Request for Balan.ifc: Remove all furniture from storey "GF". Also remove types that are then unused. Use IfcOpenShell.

First a look at what the model holds.

```python
import ifcopenshell
import ifcopenshell.util.element

model = ifcopenshell.open("Balan.ifc")
print(model.schema)
storey = next(s for s in model.by_type("IfcBuildingStorey") if s.Name == "GF")
furniture = [e for e in ifcopenshell.util.element.get_decomposition(storey) if e.is_a("IfcFurnishingElement")]
seen = {}
for e in furniture:
    element_type = ifcopenshell.util.element.get_type(e)
    name = element_type.Name if element_type not in (None, e) else None
    seen[name] = seen.get(name, 0) + 1
for name, count in sorted(seen.items(), key=str):
    print(count, "x", name)
```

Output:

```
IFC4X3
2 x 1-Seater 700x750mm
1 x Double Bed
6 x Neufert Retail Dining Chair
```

```python
import ifcopenshell
import ifcopenshell.api.root
import ifcopenshell.util.element

model = ifcopenshell.open("Balan.ifc")

storey = next(s for s in model.by_type("IfcBuildingStorey") if s.Name == "GF")
furniture = [e for e in ifcopenshell.util.element.get_decomposition(storey) if e.is_a("IfcFurnishingElement")]
types = {ifcopenshell.util.element.get_type(e) for e in furniture} - {None, *furniture}

for e in furniture:
    ifcopenshell.api.root.remove_product(model, product=e)
print(len(furniture), "removed")

unused = [t for t in types if not ifcopenshell.util.element.get_types(t)]
for t in unused:
    ifcopenshell.api.root.remove_product(model, product=t)
print(len(unused), "unused types removed")

model.write("Balan_edited.ifc")
```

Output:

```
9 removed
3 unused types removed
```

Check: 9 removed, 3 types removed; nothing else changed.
